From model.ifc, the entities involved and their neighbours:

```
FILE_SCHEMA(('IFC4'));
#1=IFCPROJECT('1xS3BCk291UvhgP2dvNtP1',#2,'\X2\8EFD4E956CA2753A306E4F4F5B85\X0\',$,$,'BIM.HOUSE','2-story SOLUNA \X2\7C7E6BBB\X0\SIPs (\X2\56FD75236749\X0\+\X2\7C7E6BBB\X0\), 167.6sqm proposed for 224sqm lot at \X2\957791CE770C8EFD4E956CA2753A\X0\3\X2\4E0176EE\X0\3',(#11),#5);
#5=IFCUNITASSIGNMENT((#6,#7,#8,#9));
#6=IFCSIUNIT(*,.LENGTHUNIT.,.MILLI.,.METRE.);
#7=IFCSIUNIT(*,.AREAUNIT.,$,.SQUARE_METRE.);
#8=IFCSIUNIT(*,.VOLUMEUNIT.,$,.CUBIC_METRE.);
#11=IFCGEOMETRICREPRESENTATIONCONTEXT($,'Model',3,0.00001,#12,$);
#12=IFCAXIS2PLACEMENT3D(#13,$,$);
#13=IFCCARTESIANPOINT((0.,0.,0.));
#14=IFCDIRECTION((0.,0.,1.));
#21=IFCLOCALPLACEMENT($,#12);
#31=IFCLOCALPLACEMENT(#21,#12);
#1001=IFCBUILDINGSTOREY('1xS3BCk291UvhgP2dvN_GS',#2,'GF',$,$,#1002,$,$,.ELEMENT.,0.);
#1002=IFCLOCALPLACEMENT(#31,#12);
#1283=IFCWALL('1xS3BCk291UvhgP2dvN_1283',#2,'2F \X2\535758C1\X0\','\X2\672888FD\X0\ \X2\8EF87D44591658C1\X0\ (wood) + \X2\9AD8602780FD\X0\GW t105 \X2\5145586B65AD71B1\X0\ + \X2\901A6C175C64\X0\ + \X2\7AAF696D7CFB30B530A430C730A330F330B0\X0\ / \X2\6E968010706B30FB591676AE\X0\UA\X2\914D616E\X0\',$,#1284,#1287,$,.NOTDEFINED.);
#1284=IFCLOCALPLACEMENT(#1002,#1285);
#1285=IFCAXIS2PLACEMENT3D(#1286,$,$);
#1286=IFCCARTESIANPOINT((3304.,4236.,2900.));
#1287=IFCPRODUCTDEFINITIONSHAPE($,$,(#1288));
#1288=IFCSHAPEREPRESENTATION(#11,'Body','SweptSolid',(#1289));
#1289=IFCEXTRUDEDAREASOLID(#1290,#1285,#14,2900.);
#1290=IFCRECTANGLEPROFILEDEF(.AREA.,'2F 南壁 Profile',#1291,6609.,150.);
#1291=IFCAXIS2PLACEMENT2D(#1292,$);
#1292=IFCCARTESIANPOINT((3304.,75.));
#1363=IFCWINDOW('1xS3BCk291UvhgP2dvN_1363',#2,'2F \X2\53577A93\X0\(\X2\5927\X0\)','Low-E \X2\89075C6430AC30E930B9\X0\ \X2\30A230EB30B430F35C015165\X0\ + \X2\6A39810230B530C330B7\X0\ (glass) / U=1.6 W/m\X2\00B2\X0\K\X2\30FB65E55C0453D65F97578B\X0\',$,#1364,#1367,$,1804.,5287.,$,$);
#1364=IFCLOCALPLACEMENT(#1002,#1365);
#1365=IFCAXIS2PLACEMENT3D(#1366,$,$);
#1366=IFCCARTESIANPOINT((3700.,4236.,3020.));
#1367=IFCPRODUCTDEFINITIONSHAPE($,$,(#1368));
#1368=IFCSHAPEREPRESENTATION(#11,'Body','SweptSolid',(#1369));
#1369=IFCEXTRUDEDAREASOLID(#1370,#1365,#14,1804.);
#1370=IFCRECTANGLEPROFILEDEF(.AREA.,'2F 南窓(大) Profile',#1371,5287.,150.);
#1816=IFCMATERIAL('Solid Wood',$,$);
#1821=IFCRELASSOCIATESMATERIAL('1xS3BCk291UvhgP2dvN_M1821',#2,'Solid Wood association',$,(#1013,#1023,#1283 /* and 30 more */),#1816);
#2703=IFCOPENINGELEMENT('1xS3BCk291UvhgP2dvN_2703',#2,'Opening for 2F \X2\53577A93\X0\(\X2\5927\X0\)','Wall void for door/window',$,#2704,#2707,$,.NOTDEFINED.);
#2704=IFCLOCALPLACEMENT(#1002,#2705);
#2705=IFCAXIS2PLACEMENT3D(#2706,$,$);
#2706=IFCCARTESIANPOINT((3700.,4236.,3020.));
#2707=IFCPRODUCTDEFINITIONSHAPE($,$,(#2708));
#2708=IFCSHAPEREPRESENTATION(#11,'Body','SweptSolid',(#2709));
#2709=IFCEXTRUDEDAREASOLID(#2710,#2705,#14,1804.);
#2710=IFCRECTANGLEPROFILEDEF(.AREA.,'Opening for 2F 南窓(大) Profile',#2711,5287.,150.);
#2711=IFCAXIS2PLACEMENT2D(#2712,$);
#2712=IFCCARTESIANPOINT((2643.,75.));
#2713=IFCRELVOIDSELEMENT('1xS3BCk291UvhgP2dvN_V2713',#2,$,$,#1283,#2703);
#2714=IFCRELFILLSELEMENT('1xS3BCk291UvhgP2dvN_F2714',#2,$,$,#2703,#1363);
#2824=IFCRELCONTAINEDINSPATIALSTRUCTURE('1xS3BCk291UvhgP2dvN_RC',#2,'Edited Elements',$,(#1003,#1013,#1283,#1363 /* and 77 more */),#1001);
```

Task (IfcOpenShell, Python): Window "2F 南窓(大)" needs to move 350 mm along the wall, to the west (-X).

```python
import ifcopenshell
import ifcopenshell.api.geometry
import ifcopenshell.util.placement

model = ifcopenshell.open("model.ifc")

window = model.by_guid("1xS3BCk291UvhgP2dvN_1363")
opening = window.FillsVoids[0].RelatingOpeningElement
wall = opening.VoidsElements[0].RelatingBuildingElement

wall_matrix = ifcopenshell.util.placement.get_local_placement(wall.ObjectPlacement)
shift = wall_matrix[:3, 0] * -350.0
before = ifcopenshell.util.placement.get_local_placement(window.ObjectPlacement)[:3, 3].copy()

# The window is not placed relative to its opening, so move both.
for product in (opening, window):
    matrix = ifcopenshell.util.placement.get_local_placement(product.ObjectPlacement)
    matrix[:3, 3] += shift
    ifcopenshell.api.geometry.edit_object_placement(model, product=product, matrix=matrix, is_si=False)

after = ifcopenshell.util.placement.get_local_placement(window.ObjectPlacement)[:3, 3]
print("window moved by", (after - before).round(3) + 0.0)

model.write("model-out.ifc")
```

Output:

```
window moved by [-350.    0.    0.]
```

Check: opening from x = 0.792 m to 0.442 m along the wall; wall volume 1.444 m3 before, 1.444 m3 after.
